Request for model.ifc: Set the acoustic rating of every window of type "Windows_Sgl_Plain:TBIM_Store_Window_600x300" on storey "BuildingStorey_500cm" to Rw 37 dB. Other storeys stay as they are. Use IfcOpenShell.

First a look at what the model holds.

```python
import ifcopenshell
import ifcopenshell.util.element

model = ifcopenshell.open("model.ifc")
print(model.schema)
storey = next(s for s in model.by_type("IfcBuildingStorey") if s.Name == "BuildingStorey_500cm")
windows = [e for e in ifcopenshell.util.element.get_decomposition(storey) if e.is_a("IfcWindow")]
seen = {}
for e in windows:
    element_type = ifcopenshell.util.element.get_type(e)
    key = (element_type.Name if element_type != e and element_type else None, ifcopenshell.util.element.get_pset(e, "Pset_WindowCommon", "AcousticRating"))
    seen[key] = seen.get(key, 0) + 1
for (name, value), count in sorted(seen.items(), key=str):
    print(count, "x", name, "|", value)
```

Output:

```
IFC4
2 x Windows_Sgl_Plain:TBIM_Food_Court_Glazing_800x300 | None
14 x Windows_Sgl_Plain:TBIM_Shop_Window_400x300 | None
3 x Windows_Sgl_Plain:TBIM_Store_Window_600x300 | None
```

```python
import ifcopenshell
import ifcopenshell.api.pset
import ifcopenshell.util.element

model = ifcopenshell.open("model.ifc")

storey = next(s for s in model.by_type("IfcBuildingStorey") if s.Name == "BuildingStorey_500cm")
windows = [e for e in ifcopenshell.util.element.get_decomposition(storey) if e.is_a("IfcWindow")]

count = 0
for e in windows:
    element_type = ifcopenshell.util.element.get_type(e)
    if element_type in (None, e) or element_type.Name != "Windows_Sgl_Plain:TBIM_Store_Window_600x300":
        continue
    # add_pset returns the element's existing set when there is one.
    pset = ifcopenshell.api.pset.add_pset(model, product=e, name="Pset_WindowCommon")
    ifcopenshell.api.pset.edit_pset(model, pset=pset, properties={"AcousticRating": "Rw 37 dB"})
    count += 1

print(count, "windows updated")

model.write("model_edited.ifc")
```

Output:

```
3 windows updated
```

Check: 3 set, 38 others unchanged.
